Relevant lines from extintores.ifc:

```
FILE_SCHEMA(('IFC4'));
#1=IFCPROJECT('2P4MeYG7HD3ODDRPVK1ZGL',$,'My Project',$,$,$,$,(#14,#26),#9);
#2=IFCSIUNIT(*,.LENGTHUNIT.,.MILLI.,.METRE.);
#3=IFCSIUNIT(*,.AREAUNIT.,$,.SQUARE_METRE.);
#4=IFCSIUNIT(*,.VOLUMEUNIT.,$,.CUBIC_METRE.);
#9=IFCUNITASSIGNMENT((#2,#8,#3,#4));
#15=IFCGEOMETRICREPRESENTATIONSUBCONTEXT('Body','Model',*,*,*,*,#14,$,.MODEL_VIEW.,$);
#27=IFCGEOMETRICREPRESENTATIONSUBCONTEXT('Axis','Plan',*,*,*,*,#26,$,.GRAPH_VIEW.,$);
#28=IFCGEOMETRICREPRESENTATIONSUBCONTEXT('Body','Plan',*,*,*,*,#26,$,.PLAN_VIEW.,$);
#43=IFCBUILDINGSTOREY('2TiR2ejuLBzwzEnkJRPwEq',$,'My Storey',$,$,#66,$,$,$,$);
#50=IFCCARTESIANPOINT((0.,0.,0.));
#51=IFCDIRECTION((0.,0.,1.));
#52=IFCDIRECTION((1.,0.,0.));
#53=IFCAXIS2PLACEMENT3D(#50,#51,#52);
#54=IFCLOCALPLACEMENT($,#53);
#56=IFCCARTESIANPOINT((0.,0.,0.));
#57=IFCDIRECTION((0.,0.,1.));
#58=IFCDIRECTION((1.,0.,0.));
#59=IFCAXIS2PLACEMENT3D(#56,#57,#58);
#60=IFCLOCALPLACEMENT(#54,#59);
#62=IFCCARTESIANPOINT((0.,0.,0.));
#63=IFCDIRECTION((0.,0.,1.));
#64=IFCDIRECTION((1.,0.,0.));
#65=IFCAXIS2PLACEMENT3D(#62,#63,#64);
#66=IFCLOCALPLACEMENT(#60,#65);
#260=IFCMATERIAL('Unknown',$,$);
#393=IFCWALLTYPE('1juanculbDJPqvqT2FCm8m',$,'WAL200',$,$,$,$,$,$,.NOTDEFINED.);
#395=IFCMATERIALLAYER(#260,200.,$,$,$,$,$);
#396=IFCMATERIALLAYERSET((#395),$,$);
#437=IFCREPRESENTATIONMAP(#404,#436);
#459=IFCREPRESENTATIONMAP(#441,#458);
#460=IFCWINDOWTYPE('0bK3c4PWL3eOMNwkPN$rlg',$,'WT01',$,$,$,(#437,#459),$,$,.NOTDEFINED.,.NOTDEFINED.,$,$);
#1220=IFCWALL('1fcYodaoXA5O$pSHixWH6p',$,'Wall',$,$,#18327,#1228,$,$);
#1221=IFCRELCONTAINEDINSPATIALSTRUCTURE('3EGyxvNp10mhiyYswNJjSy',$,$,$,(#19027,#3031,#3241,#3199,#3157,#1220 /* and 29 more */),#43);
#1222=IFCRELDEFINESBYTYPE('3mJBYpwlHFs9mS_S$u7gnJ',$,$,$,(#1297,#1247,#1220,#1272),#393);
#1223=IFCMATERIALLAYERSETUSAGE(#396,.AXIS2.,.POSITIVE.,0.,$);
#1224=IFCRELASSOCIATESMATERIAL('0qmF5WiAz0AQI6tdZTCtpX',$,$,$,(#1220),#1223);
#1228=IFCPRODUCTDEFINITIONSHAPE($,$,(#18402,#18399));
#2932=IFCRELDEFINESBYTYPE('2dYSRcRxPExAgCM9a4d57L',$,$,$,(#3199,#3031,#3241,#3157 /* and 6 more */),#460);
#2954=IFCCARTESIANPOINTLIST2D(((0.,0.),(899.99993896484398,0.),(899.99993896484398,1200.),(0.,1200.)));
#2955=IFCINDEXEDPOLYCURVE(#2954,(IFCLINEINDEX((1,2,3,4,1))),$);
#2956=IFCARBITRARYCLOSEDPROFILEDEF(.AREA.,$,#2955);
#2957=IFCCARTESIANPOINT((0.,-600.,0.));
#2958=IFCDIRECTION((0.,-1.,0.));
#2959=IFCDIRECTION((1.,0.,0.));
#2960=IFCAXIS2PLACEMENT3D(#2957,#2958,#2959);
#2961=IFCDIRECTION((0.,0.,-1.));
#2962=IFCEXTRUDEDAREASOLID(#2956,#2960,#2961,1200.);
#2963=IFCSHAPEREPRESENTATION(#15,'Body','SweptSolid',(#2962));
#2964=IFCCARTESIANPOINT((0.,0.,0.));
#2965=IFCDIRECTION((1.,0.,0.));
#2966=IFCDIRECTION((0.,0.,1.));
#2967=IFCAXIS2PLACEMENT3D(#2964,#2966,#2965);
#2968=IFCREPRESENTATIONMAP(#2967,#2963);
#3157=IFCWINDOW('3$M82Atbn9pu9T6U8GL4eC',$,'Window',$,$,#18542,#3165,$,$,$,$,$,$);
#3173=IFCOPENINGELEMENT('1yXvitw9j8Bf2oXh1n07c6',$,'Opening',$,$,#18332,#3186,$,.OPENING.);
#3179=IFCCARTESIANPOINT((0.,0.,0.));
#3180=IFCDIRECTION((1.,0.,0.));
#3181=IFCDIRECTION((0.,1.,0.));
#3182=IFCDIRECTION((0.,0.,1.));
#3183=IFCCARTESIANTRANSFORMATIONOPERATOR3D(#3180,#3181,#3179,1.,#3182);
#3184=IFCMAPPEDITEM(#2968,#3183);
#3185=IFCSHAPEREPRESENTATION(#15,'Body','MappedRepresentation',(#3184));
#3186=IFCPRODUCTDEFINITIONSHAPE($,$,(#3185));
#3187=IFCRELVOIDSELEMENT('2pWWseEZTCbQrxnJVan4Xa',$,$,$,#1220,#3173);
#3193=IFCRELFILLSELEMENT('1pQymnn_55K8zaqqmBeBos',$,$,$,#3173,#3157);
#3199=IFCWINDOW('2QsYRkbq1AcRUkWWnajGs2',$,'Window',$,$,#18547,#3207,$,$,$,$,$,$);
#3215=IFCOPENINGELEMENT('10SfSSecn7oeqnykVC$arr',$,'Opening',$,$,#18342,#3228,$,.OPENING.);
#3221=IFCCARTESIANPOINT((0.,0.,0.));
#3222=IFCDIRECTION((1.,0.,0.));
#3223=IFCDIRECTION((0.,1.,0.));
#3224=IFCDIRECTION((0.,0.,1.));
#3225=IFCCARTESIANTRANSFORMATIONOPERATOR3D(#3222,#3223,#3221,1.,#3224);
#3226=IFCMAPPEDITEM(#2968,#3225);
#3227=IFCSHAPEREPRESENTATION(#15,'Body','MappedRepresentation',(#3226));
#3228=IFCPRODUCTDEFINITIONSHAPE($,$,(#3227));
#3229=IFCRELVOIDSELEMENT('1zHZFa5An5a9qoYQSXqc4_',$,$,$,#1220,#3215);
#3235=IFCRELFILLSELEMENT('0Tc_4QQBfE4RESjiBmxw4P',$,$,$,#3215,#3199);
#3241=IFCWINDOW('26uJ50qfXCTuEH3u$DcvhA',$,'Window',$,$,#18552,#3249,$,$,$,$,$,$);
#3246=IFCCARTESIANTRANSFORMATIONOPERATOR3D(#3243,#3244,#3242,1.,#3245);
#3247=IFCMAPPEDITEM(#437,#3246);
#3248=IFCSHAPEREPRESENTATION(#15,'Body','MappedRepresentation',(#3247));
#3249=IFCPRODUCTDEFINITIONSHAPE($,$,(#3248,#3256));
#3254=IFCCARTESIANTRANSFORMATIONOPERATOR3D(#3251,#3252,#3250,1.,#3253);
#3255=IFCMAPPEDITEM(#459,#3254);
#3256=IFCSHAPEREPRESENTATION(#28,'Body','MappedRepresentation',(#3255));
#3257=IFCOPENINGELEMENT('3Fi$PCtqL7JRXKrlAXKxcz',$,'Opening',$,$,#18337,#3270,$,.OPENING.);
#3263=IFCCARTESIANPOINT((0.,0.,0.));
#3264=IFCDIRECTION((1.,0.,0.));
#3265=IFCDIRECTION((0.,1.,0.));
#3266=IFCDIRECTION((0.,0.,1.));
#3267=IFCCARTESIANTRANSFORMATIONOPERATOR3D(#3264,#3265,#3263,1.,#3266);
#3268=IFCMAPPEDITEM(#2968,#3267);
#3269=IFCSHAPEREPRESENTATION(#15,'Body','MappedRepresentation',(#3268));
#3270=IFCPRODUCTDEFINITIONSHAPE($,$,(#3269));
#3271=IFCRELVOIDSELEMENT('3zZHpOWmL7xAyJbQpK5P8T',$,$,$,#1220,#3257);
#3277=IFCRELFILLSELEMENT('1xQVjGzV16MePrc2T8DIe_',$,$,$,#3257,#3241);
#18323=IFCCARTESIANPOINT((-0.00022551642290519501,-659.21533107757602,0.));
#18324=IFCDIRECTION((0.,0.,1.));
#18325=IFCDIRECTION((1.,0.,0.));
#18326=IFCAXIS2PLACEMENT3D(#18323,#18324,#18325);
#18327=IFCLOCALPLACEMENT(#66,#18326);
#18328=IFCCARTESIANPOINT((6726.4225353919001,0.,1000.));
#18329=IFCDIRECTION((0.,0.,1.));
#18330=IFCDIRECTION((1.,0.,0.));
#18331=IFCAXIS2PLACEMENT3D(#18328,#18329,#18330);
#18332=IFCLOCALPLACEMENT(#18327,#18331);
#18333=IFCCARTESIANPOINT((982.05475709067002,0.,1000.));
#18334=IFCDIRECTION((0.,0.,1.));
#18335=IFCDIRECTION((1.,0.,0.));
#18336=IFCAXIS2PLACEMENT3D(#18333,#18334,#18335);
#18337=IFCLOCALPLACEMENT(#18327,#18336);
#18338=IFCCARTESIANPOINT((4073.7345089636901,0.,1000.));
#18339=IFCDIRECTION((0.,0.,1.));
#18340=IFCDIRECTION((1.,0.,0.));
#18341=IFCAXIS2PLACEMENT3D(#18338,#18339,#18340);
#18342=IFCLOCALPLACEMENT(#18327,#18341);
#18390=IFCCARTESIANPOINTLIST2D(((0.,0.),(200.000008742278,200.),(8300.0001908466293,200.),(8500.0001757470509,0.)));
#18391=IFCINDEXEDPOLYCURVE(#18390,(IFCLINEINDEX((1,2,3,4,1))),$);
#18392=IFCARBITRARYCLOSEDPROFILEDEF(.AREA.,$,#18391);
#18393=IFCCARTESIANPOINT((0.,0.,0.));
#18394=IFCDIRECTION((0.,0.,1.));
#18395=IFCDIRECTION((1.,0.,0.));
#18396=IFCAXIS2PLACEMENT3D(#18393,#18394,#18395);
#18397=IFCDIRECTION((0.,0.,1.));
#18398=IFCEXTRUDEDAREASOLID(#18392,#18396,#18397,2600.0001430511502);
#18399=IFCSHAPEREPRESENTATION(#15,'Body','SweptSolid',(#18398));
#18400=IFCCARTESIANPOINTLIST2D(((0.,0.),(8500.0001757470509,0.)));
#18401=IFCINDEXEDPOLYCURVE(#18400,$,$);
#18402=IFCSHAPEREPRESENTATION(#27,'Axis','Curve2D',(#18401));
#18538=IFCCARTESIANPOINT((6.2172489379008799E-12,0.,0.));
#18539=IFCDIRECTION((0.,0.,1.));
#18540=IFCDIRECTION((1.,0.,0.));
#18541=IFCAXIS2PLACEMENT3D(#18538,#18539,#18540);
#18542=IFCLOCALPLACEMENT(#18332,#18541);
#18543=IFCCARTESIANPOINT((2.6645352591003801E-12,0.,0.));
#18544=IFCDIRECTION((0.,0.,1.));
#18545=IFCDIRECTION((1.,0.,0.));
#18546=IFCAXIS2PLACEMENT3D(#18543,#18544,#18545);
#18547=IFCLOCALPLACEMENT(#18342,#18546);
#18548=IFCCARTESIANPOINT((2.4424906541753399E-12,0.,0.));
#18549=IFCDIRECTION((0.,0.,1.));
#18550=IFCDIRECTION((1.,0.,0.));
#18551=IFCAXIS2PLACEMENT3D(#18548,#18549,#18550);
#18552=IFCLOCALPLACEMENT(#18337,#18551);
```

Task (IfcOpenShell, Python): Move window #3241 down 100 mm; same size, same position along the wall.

```python
import numpy as np
import ifcopenshell
import ifcopenshell.api.geometry
import ifcopenshell.util.placement
import ifcopenshell.util.unit

model = ifcopenshell.open("extintores.ifc")
unit_scale = ifcopenshell.util.unit.calculate_unit_scale(model)

window = model.by_guid("26uJ50qfXCTuEH3u$DcvhA")
opening = window.FillsVoids[0].RelatingOpeningElement
dz = -100.0

shift = np.array([0.0, 0.0, dz])
# The window is placed relative to its opening, so it follows when the opening moves.
matrix = ifcopenshell.util.placement.get_local_placement(opening.ObjectPlacement)
matrix[:3, 3] += shift
ifcopenshell.api.geometry.edit_object_placement(
    model, product=opening, matrix=matrix, is_si=False, should_transform_children=True
)

print(f"moved by {dz * unit_scale:+.3f} m")

model.write("extintores_edited.ifc")
```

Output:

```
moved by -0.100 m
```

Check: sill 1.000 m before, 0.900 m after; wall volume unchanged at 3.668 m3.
